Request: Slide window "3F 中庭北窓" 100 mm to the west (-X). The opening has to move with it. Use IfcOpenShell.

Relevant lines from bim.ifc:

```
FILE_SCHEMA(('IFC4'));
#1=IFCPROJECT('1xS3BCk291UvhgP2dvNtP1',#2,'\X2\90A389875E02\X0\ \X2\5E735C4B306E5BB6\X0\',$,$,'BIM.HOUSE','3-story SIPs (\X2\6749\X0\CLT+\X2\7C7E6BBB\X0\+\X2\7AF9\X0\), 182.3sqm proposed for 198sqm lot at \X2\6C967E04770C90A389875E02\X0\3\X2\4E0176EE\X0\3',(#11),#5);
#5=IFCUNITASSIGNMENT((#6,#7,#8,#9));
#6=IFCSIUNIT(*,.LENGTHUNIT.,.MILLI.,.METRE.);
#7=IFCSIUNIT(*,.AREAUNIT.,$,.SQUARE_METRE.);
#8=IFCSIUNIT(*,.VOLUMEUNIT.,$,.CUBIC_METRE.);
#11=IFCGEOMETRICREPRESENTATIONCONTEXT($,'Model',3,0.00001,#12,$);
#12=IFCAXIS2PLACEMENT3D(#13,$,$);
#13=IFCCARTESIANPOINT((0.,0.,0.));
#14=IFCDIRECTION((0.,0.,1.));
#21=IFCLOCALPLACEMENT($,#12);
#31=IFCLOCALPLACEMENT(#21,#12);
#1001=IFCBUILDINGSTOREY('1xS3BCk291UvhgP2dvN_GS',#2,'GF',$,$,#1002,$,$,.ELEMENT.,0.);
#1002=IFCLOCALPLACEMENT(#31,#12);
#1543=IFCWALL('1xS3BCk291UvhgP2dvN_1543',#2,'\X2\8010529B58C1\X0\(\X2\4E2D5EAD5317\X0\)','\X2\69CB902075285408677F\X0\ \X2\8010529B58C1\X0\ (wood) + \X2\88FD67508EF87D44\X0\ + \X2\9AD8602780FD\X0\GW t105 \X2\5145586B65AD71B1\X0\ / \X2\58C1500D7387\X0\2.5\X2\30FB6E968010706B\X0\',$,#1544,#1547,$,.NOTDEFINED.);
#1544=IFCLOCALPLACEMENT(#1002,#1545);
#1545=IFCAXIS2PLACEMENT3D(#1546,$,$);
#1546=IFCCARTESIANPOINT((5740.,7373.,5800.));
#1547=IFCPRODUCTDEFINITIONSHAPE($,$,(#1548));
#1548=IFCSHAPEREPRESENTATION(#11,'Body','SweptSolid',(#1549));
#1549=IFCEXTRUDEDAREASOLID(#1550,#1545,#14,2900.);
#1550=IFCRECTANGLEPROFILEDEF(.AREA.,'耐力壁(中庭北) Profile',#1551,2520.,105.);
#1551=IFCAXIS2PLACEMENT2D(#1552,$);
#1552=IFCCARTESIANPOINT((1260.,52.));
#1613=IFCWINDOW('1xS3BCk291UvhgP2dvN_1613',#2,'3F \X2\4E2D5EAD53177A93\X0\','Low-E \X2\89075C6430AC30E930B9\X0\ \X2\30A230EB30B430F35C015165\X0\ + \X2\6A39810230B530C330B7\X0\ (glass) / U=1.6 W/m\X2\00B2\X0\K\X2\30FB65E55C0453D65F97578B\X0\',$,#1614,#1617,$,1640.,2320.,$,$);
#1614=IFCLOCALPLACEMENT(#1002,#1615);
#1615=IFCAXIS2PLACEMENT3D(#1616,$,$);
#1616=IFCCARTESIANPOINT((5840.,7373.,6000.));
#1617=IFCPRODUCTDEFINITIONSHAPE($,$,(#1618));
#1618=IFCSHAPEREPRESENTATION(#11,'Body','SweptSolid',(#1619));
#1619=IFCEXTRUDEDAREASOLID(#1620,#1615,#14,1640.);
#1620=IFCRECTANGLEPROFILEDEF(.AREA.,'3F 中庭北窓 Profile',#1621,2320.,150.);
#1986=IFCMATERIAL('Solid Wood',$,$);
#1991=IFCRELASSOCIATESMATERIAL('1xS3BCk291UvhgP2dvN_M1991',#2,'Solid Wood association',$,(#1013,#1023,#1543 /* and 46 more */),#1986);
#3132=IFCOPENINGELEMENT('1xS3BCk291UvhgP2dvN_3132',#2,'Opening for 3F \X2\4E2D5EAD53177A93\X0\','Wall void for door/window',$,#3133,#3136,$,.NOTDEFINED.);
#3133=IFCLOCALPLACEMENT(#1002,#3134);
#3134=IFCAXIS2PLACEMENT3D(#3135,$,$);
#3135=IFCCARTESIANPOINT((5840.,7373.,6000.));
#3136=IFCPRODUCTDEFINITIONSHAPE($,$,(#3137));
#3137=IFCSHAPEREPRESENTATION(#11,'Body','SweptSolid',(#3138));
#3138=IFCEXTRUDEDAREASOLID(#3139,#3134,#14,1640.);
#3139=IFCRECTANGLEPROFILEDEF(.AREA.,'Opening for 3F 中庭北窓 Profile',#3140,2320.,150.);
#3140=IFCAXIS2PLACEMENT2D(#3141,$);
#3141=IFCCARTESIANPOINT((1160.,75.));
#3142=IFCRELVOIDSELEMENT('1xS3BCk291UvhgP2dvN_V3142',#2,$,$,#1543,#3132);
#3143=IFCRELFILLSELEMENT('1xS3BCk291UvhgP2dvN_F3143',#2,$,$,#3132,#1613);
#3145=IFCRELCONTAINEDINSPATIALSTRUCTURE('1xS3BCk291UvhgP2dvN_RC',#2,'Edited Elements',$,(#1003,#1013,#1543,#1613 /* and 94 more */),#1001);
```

```python
import ifcopenshell
import ifcopenshell.api.geometry
import ifcopenshell.util.placement

model = ifcopenshell.open("bim.ifc")

window = model.by_guid("1xS3BCk291UvhgP2dvN_1613")
opening = window.FillsVoids[0].RelatingOpeningElement
wall = opening.VoidsElements[0].RelatingBuildingElement

wall_matrix = ifcopenshell.util.placement.get_local_placement(wall.ObjectPlacement)
shift = wall_matrix[:3, 0] * -100.0
before = ifcopenshell.util.placement.get_local_placement(window.ObjectPlacement)[:3, 3].copy()

# The window is not placed relative to its opening, so move both.
for product in (opening, window):
    matrix = ifcopenshell.util.placement.get_local_placement(product.ObjectPlacement)
    matrix[:3, 3] += shift
    ifcopenshell.api.geometry.edit_object_placement(model, product=product, matrix=matrix, is_si=False)

after = ifcopenshell.util.placement.get_local_placement(window.ObjectPlacement)[:3, 3]
print("window moved by", (after - before).round(3) + 0.0)

model.write("bim_updated.ifc")
```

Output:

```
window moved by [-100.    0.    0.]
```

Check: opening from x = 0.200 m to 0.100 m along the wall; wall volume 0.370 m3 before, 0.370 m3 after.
